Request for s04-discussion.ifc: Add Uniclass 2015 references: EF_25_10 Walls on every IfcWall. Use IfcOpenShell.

First a look at what the model holds.

```python
import ifcopenshell

model = ifcopenshell.open("s04-discussion.ifc")
print(model.schema)
print("classifications:", [c.Name for c in model.by_type("IfcClassification")])
for ifc_class in ("IfcDoor", "IfcRoof", "IfcStair", "IfcWall", "IfcWindow"):
    print(ifc_class, len(model.by_type(ifc_class)))
```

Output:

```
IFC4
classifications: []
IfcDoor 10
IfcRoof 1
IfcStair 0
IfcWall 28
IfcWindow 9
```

```python
import ifcopenshell
import ifcopenshell.api.classification

model = ifcopenshell.open("s04-discussion.ifc")

system = ifcopenshell.api.classification.add_classification(model, classification="Uniclass 2015")

codes = {
    "IfcWall": ("EF_25_10", "Walls"),
}
for ifc_class, (code, name) in codes.items():
    products = model.by_type(ifc_class)
    ifcopenshell.api.classification.add_reference(
        model, products=products, classification=system, identification=code, name=name
    )
    print(code, len(products))

model.write("s04-discussion_updated.ifc")
```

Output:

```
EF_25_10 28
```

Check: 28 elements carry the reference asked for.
